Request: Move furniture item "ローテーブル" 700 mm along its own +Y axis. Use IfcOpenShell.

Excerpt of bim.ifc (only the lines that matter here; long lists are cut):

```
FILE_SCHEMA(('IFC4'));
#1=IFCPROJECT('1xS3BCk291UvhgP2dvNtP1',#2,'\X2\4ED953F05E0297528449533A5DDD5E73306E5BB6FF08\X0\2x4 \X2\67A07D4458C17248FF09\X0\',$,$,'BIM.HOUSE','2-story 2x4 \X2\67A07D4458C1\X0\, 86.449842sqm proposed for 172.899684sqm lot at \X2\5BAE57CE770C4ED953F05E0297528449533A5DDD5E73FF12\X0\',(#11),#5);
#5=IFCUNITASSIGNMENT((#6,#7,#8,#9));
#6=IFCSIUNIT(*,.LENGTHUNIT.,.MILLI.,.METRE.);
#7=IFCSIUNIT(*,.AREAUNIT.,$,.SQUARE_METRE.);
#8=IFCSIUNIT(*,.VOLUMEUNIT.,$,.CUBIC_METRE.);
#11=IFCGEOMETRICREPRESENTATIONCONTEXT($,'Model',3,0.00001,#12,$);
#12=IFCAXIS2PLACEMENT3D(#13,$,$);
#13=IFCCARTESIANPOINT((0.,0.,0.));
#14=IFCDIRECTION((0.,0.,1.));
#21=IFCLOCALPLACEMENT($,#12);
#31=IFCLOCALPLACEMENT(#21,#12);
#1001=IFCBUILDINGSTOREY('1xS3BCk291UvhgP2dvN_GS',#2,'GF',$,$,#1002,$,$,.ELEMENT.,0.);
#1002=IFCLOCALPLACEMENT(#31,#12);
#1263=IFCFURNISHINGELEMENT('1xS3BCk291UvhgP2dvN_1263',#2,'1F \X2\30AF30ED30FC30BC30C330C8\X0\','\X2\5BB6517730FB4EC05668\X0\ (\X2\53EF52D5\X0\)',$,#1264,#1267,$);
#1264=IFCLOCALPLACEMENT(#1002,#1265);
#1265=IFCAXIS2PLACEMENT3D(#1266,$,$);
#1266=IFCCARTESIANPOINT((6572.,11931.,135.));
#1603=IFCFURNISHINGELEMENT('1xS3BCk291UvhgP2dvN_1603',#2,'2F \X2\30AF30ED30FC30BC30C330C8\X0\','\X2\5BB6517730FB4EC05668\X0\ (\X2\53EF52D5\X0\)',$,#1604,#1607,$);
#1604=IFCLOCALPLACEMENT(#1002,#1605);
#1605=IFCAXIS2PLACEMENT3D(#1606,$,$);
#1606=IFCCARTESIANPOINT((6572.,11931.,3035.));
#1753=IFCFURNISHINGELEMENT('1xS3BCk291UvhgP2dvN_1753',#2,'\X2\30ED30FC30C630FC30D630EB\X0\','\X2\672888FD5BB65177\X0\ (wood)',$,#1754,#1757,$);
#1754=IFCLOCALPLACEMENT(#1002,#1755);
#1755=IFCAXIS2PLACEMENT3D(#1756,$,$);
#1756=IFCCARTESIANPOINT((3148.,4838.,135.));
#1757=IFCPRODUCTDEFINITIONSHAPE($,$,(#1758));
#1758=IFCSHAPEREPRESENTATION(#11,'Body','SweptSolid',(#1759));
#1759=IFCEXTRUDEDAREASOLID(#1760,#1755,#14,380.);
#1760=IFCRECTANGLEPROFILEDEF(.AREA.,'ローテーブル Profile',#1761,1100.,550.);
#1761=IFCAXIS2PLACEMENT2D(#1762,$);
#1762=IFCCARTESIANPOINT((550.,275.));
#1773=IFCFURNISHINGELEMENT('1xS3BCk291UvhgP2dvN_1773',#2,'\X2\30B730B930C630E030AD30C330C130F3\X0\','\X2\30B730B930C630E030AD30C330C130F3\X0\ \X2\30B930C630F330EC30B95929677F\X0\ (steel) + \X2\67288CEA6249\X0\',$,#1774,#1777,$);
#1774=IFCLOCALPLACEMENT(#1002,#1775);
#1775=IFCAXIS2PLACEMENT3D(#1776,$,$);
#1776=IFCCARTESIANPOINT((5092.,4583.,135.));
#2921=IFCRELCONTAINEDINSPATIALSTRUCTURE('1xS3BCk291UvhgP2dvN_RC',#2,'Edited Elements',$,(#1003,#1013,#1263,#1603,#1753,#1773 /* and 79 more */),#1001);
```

```python
import ifcopenshell
import ifcopenshell.api.geometry
import ifcopenshell.util.placement

model = ifcopenshell.open("bim.ifc")

item = model.by_guid("1xS3BCk291UvhgP2dvN_1753")
matrix = ifcopenshell.util.placement.get_local_placement(item.ObjectPlacement)
matrix[:3, 3] += matrix[:3, 1] * 700.0
ifcopenshell.api.geometry.edit_object_placement(model, product=item, matrix=matrix, is_si=False)

print(ifcopenshell.util.placement.get_local_placement(item.ObjectPlacement).round(3) + 0.0)

model.write("bim_rev.ifc")
```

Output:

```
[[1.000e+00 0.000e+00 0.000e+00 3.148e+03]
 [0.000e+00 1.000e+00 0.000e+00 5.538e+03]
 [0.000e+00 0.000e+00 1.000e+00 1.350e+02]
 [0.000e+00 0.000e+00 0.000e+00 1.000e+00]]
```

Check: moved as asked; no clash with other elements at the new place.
